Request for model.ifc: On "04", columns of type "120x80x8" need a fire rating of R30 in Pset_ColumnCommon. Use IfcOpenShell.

First a look at what the model holds.

```python
import ifcopenshell
import ifcopenshell.util.element

model = ifcopenshell.open("model.ifc")
print(model.schema)
storey = next(s for s in model.by_type("IfcBuildingStorey") if s.Name == "04")
columns = [e for e in ifcopenshell.util.element.get_decomposition(storey) if e.is_a("IfcColumn")]
seen = {}
for e in columns:
    element_type = ifcopenshell.util.element.get_type(e)
    key = (element_type.Name if element_type != e and element_type else None, ifcopenshell.util.element.get_pset(e, "Pset_ColumnCommon", "FireRating"))
    seen[key] = seen.get(key, 0) + 1
for (name, value), count in sorted(seen.items(), key=str):
    print(count, "x", name, "|", value)
```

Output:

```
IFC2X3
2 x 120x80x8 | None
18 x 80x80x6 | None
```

```python
import ifcopenshell
import ifcopenshell.api.pset
import ifcopenshell.util.element

model = ifcopenshell.open("model.ifc")

storey = next(s for s in model.by_type("IfcBuildingStorey") if s.Name == "04")
columns = [e for e in ifcopenshell.util.element.get_decomposition(storey) if e.is_a("IfcColumn")]

count = 0
for e in columns:
    element_type = ifcopenshell.util.element.get_type(e)
    if element_type in (None, e) or element_type.Name != "120x80x8":
        continue
    # add_pset returns the element's existing set when there is one.
    pset = ifcopenshell.api.pset.add_pset(model, product=e, name="Pset_ColumnCommon")
    ifcopenshell.api.pset.edit_pset(model, pset=pset, properties={"FireRating": "R30"})
    count += 1

print(count, "columns updated")

model.write("model_updated.ifc")
```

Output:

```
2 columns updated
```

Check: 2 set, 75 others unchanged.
